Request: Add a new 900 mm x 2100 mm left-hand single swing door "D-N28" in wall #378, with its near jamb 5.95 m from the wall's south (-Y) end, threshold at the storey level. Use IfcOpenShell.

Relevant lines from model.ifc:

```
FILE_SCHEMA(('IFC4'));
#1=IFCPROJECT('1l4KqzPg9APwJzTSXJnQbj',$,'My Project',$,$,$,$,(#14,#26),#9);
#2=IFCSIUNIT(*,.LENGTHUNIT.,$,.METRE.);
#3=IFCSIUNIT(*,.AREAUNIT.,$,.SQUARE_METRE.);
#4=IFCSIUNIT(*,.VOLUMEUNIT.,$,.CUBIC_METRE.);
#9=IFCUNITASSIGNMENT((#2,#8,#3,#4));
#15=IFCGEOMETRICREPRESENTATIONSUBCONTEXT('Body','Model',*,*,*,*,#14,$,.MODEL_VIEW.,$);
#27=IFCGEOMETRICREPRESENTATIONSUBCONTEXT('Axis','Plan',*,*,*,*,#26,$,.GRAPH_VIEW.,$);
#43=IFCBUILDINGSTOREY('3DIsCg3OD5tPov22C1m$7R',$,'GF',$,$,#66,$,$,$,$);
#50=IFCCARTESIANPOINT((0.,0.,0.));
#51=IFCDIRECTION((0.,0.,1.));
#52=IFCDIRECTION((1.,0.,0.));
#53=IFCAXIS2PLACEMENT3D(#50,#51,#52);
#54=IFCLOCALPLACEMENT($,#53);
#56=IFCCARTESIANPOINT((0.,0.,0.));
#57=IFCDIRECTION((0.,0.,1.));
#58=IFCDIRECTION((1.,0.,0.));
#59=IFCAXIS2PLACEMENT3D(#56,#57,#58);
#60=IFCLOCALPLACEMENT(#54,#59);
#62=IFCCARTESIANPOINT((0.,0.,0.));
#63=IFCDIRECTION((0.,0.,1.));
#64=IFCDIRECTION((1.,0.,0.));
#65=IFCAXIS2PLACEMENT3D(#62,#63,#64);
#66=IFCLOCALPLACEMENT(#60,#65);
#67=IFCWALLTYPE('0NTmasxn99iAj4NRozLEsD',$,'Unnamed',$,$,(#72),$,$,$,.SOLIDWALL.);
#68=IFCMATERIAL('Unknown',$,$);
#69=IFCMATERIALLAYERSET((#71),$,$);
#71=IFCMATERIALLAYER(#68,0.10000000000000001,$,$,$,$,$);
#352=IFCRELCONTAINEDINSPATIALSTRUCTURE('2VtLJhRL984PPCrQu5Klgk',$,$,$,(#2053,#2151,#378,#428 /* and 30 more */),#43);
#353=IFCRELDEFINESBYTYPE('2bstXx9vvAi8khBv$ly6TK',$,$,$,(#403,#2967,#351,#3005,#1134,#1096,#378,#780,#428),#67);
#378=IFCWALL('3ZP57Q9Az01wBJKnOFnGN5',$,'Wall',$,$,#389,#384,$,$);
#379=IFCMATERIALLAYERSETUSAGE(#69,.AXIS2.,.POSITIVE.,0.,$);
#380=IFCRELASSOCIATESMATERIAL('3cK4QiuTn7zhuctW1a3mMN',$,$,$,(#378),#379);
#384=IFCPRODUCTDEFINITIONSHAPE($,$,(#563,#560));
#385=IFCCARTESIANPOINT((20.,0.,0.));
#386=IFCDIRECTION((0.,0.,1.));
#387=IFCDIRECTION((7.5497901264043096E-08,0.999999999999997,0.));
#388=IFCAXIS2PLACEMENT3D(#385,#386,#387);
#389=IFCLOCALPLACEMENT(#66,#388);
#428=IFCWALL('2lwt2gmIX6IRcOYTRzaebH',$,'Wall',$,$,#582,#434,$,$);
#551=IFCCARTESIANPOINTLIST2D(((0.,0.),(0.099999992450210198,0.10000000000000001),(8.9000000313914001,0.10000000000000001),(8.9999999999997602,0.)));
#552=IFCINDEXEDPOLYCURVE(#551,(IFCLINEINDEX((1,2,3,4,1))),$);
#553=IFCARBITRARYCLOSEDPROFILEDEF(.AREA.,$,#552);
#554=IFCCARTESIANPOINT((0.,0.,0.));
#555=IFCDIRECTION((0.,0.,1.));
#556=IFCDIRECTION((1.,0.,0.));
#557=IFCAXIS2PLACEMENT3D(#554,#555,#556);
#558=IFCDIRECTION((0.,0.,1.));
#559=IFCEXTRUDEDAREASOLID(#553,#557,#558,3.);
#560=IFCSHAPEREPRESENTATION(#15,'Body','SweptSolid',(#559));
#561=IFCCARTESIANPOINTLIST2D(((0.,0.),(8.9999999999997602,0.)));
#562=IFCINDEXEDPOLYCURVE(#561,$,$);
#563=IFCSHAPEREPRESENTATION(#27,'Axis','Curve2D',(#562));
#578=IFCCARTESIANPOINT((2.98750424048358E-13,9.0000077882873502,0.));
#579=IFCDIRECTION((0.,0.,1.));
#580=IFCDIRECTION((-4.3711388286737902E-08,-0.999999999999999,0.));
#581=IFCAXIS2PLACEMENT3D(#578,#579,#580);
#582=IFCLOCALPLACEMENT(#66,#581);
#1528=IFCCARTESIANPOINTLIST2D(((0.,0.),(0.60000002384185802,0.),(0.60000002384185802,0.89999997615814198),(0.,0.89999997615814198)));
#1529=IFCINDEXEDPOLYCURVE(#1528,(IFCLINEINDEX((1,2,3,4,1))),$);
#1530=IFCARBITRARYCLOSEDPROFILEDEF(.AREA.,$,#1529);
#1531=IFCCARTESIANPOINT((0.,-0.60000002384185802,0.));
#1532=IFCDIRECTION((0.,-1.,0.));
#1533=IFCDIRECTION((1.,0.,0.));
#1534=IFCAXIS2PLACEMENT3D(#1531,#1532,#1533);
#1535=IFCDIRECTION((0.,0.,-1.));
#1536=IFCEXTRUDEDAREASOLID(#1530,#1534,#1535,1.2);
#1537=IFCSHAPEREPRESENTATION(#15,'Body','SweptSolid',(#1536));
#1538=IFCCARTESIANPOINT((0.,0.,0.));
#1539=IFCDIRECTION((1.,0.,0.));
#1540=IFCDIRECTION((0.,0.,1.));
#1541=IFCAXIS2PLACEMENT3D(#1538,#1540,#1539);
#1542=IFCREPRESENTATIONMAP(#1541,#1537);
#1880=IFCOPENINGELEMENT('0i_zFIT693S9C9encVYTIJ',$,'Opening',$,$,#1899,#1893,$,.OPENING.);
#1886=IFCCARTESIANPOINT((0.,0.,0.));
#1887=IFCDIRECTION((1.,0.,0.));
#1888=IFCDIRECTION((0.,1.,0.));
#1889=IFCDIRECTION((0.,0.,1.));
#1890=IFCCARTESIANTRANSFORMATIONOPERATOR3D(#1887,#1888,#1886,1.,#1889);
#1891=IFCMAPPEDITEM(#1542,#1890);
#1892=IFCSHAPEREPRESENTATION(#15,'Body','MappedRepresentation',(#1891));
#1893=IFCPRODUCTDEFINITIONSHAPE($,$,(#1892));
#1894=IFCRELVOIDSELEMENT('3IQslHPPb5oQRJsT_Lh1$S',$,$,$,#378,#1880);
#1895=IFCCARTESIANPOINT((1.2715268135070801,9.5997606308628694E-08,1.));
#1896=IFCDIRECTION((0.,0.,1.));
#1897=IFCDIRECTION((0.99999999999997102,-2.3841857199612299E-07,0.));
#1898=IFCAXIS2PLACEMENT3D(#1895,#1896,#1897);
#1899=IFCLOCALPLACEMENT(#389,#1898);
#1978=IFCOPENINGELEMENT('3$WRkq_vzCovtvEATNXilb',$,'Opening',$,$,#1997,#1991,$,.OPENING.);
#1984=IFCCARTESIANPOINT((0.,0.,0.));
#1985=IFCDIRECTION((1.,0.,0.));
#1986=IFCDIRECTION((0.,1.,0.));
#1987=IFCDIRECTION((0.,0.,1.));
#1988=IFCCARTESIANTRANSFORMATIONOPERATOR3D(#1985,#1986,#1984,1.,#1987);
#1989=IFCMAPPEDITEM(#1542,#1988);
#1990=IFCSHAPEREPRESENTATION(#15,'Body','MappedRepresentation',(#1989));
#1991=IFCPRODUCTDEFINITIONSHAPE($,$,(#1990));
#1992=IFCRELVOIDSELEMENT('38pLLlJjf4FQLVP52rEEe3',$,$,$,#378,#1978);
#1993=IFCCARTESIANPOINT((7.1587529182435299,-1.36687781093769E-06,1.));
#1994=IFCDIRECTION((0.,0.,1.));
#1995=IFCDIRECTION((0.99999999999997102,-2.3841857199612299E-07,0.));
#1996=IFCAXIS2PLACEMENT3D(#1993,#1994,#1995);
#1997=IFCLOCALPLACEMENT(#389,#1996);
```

```python
import numpy as np
import ifcopenshell
import ifcopenshell.api.feature
import ifcopenshell.api.geometry
import ifcopenshell.api.root
import ifcopenshell.api.spatial
import ifcopenshell.geom
import ifcopenshell.util.element
import ifcopenshell.util.placement
import ifcopenshell.util.representation
import ifcopenshell.util.shape
import ifcopenshell.util.unit

model = ifcopenshell.open("model.ifc")
unit_scale = ifcopenshell.util.unit.calculate_unit_scale(model)
settings = ifcopenshell.geom.settings()


def volume(element):
    """Net volume in cubic metres, openings subtracted."""
    shape = ifcopenshell.geom.create_shape(settings, element)
    return ifcopenshell.util.shape.get_volume(shape.geometry)


wall = model.by_guid("3ZP57Q9Az01wBJKnOFnGN5")
storey = ifcopenshell.util.element.get_container(wall, ifc_class="IfcBuildingStorey")
context = ifcopenshell.util.representation.get_context(model, "Model", "Body", "MODEL_VIEW")
before = volume(wall)

width, height, from_end, sill = 0.9, 2.1, 5.95, 0.0  # metres

# The wall runs along its own X axis, and the end named is its -X end.
wall_shape = ifcopenshell.geom.create_shape(settings, wall)
x, y, z = ifcopenshell.util.shape.get_vertices(wall_shape.geometry).T
start = x.min() + from_end
face, thickness = float(y.min()), float(y.max() - y.min())
wall_matrix = ifcopenshell.util.placement.get_local_placement(wall.ObjectPlacement)
level = ifcopenshell.util.placement.get_local_placement(storey.ObjectPlacement)[2, 3]


def in_wall(x, y):
    """Placement at x, y metres in the wall's axes, at sill height."""
    matrix = wall_matrix.copy()
    matrix[:, 3] = wall_matrix @ np.array([x / unit_scale, y / unit_scale, 0.0, 1.0])
    matrix[2, 3] = level + sill / unit_scale
    return matrix


# Opening: a box that overshoots both wall faces by 50 mm.
opening = ifcopenshell.api.root.create_entity(model, ifc_class="IfcOpeningElement", predefined_type="OPENING")
box = ifcopenshell.api.geometry.add_wall_representation(
    model, context=context, length=width, height=height, thickness=thickness + 0.1
)
ifcopenshell.api.geometry.assign_representation(model, product=opening, representation=box)
ifcopenshell.api.geometry.edit_object_placement(model, product=opening, matrix=in_wall(start, face - 0.05), is_si=False)
ifcopenshell.api.feature.add_feature(model, feature=opening, element=wall)

door = ifcopenshell.api.root.create_entity(model, ifc_class="IfcDoor", name="D-N28", predefined_type="DOOR")
door.OverallWidth, door.OverallHeight = width / unit_scale, height / unit_scale
door.OperationType = "SINGLE_SWING_LEFT"
body = ifcopenshell.api.geometry.add_door_representation(
    model,
    context=context,
    overall_width=door.OverallWidth,
    overall_height=door.OverallHeight,
    operation_type="SINGLE_SWING_LEFT",
    lining_properties={"LiningDepth": thickness / unit_scale, "ThresholdDepth": thickness / unit_scale},
)
ifcopenshell.api.geometry.assign_representation(model, product=door, representation=body)
ifcopenshell.api.spatial.assign_container(model, products=[door], relating_structure=storey)
ifcopenshell.api.feature.add_filling(model, opening=opening, element=door)

# The lining spans the wall, so the door starts at the wall face.
ifcopenshell.api.geometry.edit_object_placement(model, product=door, matrix=in_wall(start, face), is_si=False)

after = volume(wall)

print(f"wall volume {before:.3f} -> {after:.3f} m3")

model.write("model_updated.ifc")
```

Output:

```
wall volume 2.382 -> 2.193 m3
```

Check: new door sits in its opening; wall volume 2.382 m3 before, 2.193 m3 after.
